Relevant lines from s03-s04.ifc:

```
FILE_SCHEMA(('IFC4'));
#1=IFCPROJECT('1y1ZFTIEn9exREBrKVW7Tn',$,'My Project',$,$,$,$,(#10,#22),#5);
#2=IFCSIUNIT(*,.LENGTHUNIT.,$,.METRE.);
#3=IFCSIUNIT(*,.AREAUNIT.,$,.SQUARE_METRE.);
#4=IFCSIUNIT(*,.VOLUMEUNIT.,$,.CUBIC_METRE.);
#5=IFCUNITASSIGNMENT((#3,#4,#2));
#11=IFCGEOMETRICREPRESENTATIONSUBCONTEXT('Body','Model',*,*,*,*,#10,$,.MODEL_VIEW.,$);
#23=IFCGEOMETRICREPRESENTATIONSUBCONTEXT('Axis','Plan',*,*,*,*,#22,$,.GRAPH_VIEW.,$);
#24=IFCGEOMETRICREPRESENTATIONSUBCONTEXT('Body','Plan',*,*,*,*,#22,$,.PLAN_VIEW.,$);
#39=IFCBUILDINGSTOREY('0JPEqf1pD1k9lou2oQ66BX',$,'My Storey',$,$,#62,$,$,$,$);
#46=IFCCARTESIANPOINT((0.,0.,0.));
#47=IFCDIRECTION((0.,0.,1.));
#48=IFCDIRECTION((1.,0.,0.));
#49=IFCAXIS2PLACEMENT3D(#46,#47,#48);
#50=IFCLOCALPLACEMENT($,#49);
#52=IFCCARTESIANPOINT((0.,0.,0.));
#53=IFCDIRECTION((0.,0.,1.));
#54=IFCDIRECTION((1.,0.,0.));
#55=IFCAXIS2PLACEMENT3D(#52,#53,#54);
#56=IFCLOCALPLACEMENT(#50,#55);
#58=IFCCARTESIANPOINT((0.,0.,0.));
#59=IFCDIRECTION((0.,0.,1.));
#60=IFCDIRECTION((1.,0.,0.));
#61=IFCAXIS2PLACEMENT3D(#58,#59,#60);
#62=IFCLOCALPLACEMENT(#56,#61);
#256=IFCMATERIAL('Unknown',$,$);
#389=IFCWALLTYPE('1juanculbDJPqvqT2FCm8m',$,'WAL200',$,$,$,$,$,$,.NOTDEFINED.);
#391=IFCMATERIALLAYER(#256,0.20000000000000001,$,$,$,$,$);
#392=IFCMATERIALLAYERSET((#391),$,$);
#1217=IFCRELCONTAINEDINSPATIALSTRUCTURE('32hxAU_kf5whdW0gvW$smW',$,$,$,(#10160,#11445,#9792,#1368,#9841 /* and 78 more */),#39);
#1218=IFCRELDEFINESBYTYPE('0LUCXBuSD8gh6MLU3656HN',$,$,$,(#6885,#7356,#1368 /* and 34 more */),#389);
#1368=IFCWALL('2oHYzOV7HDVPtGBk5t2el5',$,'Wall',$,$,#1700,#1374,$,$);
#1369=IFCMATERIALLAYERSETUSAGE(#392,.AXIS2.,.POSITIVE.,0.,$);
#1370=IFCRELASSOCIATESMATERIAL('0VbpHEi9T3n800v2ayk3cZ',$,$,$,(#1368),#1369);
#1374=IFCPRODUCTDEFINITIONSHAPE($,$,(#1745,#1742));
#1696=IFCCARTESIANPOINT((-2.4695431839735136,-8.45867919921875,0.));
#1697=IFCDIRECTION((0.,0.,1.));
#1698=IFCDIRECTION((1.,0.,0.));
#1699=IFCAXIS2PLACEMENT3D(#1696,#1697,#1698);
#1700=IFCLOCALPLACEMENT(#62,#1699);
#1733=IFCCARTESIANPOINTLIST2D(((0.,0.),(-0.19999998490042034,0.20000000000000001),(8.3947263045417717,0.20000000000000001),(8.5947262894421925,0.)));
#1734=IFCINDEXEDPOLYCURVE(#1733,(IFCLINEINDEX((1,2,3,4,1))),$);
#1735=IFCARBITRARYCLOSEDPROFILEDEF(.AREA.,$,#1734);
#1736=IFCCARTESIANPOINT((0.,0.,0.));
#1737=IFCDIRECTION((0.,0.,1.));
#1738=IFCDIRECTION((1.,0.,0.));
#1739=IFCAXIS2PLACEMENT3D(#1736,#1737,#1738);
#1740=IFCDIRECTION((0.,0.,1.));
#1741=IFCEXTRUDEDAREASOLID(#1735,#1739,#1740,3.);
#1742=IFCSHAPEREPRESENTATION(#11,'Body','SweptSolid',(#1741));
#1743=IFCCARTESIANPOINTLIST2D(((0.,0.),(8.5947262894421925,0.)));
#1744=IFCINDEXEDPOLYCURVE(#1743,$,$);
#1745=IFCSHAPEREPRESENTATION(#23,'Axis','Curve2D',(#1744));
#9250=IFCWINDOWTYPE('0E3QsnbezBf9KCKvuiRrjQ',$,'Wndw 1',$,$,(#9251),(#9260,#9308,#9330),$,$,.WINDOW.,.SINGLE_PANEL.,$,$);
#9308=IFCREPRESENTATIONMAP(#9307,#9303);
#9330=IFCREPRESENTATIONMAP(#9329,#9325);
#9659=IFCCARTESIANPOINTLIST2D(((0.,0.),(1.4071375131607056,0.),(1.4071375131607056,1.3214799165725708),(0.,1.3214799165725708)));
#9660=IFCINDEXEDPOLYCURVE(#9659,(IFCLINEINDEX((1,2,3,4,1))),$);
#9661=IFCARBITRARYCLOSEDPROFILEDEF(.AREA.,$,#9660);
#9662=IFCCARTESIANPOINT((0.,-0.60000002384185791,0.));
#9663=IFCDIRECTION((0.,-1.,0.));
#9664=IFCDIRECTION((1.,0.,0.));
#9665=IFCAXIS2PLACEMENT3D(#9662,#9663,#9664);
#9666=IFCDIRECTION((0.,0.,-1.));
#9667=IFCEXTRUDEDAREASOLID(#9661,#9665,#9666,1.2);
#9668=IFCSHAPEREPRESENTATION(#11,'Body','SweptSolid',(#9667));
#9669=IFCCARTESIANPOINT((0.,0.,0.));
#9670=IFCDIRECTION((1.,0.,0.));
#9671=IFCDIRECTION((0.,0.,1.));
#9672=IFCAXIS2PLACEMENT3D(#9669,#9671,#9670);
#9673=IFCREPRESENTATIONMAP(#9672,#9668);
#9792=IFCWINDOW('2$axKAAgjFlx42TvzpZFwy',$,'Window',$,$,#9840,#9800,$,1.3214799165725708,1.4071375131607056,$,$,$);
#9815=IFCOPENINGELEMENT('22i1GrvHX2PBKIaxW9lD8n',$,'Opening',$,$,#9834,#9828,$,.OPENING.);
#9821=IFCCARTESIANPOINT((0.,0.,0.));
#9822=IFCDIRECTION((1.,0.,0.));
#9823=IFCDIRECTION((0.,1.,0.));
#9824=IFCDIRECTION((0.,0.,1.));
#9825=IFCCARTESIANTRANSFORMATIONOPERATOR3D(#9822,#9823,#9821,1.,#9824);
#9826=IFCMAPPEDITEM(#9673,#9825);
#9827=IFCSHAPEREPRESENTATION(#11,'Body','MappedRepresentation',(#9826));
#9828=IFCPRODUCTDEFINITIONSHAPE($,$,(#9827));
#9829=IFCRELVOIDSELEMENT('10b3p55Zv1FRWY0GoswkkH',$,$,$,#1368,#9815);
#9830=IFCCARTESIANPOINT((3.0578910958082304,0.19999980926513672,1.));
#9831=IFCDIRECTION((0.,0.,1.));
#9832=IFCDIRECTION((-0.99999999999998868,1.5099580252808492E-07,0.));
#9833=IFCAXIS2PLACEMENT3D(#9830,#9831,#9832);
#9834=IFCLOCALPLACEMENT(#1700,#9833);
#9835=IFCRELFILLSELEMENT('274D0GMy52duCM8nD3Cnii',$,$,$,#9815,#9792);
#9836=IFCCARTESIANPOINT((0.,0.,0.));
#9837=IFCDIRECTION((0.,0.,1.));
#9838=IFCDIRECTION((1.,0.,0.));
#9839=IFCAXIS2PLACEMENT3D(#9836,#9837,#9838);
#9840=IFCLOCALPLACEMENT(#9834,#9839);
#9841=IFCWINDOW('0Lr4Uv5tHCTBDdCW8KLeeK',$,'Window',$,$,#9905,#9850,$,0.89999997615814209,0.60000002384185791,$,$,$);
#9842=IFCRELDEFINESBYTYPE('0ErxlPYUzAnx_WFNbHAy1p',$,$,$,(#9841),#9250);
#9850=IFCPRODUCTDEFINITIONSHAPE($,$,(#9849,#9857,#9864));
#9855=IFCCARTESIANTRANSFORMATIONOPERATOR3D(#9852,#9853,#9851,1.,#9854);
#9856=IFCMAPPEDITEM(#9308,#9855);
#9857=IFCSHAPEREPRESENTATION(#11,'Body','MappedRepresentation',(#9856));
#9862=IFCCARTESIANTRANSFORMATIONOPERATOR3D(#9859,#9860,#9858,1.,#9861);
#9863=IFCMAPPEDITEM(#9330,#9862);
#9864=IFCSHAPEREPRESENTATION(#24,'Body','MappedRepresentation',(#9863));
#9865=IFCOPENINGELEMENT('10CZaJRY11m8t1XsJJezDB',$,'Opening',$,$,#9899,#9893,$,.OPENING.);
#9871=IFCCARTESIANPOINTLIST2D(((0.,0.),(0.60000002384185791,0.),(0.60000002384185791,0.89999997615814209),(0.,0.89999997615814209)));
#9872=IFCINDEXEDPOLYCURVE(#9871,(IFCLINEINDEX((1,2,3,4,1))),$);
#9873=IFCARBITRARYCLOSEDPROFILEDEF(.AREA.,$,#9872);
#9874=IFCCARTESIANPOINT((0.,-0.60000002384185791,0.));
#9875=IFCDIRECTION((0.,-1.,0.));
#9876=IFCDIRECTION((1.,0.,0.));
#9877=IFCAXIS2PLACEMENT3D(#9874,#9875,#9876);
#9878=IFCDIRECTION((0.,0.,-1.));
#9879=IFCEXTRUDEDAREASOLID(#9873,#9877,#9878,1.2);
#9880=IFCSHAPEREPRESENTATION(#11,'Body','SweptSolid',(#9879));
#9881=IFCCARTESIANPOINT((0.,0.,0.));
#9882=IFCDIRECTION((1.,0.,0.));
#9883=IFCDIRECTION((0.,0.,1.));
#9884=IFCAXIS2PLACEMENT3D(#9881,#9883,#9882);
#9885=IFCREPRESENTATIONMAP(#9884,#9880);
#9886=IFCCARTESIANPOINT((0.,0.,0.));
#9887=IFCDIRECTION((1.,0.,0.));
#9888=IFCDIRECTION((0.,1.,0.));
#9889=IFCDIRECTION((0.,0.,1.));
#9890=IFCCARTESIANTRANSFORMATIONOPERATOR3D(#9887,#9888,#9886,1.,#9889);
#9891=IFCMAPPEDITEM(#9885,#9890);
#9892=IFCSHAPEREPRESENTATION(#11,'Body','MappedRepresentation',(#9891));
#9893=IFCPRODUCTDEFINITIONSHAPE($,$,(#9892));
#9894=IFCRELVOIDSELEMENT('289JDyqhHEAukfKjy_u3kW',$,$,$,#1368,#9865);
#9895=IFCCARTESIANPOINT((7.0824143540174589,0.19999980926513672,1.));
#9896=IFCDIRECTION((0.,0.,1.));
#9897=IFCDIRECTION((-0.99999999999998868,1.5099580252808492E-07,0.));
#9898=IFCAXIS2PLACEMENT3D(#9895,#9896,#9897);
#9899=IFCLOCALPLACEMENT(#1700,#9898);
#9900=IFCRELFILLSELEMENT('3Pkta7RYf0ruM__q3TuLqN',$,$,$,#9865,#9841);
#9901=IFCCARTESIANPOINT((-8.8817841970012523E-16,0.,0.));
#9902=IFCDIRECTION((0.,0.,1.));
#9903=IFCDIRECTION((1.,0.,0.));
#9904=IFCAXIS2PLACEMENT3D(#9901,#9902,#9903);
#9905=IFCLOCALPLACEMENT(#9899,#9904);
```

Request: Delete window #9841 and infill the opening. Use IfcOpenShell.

```python
import ifcopenshell
import ifcopenshell.api.feature
import ifcopenshell.api.root
import ifcopenshell.geom
import ifcopenshell.util.shape

model = ifcopenshell.open("s03-s04.ifc")
settings = ifcopenshell.geom.settings()


def volume(element):
    """Net volume in cubic metres, openings subtracted."""
    shape = ifcopenshell.geom.create_shape(settings, element)
    return ifcopenshell.util.shape.get_volume(shape.geometry)


window = model.by_guid("0Lr4Uv5tHCTBDdCW8KLeeK")
opening = window.FillsVoids[0].RelatingOpeningElement
wall = opening.VoidsElements[0].RelatingBuildingElement
before = volume(wall)

ifcopenshell.api.root.remove_product(model, product=window)
ifcopenshell.api.feature.remove_feature(model, feature=opening)

after = volume(wall)

print(f"wall volume {before:.3f} -> {after:.3f} m3")

model.write("s03-s04_edited.ifc")
```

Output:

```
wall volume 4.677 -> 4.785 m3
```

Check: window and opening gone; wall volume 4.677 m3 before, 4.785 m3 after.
